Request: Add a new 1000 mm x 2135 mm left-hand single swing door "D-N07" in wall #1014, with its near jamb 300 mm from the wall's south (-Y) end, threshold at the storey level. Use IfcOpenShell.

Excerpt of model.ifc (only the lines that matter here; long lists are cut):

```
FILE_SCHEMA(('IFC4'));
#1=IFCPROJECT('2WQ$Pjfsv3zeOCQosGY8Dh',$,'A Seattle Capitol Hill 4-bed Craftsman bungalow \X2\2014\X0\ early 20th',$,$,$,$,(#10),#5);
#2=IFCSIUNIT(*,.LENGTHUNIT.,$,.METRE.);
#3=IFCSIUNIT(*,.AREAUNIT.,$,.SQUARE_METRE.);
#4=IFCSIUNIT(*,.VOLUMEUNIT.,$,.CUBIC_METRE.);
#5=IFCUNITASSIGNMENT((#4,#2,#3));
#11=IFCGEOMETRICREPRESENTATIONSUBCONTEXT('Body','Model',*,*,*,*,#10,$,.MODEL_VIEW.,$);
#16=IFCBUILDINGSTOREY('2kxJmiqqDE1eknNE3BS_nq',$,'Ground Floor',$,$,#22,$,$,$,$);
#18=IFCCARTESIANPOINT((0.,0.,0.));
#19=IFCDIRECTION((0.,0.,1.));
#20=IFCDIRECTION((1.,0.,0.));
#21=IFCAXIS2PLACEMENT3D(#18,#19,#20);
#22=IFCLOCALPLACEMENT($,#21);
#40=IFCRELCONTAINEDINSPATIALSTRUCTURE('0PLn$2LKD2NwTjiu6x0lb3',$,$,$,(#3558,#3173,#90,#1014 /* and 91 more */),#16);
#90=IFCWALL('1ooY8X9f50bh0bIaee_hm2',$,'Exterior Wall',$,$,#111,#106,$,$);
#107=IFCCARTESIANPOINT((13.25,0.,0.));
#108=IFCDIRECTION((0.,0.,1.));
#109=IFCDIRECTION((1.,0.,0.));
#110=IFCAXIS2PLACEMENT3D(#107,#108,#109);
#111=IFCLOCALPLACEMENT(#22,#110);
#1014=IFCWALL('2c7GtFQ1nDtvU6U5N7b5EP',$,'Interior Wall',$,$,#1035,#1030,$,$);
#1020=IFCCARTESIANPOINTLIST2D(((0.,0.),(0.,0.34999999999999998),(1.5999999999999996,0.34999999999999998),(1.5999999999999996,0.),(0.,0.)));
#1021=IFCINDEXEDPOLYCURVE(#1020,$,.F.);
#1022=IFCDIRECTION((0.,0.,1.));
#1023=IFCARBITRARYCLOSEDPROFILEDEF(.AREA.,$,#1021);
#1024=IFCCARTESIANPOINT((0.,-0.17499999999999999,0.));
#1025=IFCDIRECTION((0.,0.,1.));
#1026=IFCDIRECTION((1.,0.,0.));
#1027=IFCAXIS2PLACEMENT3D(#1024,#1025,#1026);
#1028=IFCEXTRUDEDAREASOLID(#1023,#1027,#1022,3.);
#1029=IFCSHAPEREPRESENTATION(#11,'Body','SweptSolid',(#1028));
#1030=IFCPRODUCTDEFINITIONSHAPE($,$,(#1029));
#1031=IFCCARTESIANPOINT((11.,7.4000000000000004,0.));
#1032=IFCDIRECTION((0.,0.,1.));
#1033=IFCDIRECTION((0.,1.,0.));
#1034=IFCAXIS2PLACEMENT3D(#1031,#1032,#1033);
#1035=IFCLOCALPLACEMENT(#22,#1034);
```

```python
import numpy as np
import ifcopenshell
import ifcopenshell.api.feature
import ifcopenshell.api.geometry
import ifcopenshell.api.root
import ifcopenshell.api.spatial
import ifcopenshell.geom
import ifcopenshell.util.element
import ifcopenshell.util.placement
import ifcopenshell.util.representation
import ifcopenshell.util.shape
import ifcopenshell.util.unit

model = ifcopenshell.open("model.ifc")
unit_scale = ifcopenshell.util.unit.calculate_unit_scale(model)
settings = ifcopenshell.geom.settings()


def volume(element):
    """Net volume in cubic metres, openings subtracted."""
    shape = ifcopenshell.geom.create_shape(settings, element)
    return ifcopenshell.util.shape.get_volume(shape.geometry)


wall = model.by_id(1014)
storey = ifcopenshell.util.element.get_container(wall, ifc_class="IfcBuildingStorey")
context = ifcopenshell.util.representation.get_context(model, "Model", "Body", "MODEL_VIEW")
before = volume(wall)

width, height, from_end, sill = 1, 2.135, 0.3, 0.0  # metres

# The wall runs along its own X axis, and the end named is its -X end.
wall_shape = ifcopenshell.geom.create_shape(settings, wall)
x, y, z = ifcopenshell.util.shape.get_vertices(wall_shape.geometry).T
start = x.min() + from_end
face, thickness = float(y.min()), float(y.max() - y.min())
wall_matrix = ifcopenshell.util.placement.get_local_placement(wall.ObjectPlacement)
level = ifcopenshell.util.placement.get_local_placement(storey.ObjectPlacement)[2, 3]


def in_wall(x, y):
    """Placement at x, y metres in the wall's axes, at sill height."""
    matrix = wall_matrix.copy()
    matrix[:, 3] = wall_matrix @ np.array([x / unit_scale, y / unit_scale, 0.0, 1.0])
    matrix[2, 3] = level + sill / unit_scale
    return matrix


# Opening: a box that overshoots both wall faces by 50 mm.
opening = ifcopenshell.api.root.create_entity(model, ifc_class="IfcOpeningElement", predefined_type="OPENING")
box = ifcopenshell.api.geometry.add_wall_representation(
    model, context=context, length=width, height=height, thickness=thickness + 0.1
)
ifcopenshell.api.geometry.assign_representation(model, product=opening, representation=box)
ifcopenshell.api.geometry.edit_object_placement(model, product=opening, matrix=in_wall(start, face - 0.05), is_si=False)
ifcopenshell.api.feature.add_feature(model, feature=opening, element=wall)

door = ifcopenshell.api.root.create_entity(model, ifc_class="IfcDoor", name="D-N07", predefined_type="DOOR")
door.OverallWidth, door.OverallHeight = width / unit_scale, height / unit_scale
door.OperationType = "SINGLE_SWING_LEFT"
body = ifcopenshell.api.geometry.add_door_representation(
    model,
    context=context,
    overall_width=door.OverallWidth,
    overall_height=door.OverallHeight,
    operation_type="SINGLE_SWING_LEFT",
    lining_properties={"LiningDepth": thickness / unit_scale, "ThresholdDepth": thickness / unit_scale},
)
ifcopenshell.api.geometry.assign_representation(model, product=door, representation=body)
ifcopenshell.api.spatial.assign_container(model, products=[door], relating_structure=storey)
ifcopenshell.api.feature.add_filling(model, opening=opening, element=door)

# The lining spans the wall, so the door starts at the wall face.
ifcopenshell.api.geometry.edit_object_placement(model, product=door, matrix=in_wall(start, face), is_si=False)

after = volume(wall)

print(f"wall volume {before:.3f} -> {after:.3f} m3")

model.write("model-out.ifc")
```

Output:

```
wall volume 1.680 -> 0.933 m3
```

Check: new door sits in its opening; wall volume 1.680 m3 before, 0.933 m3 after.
